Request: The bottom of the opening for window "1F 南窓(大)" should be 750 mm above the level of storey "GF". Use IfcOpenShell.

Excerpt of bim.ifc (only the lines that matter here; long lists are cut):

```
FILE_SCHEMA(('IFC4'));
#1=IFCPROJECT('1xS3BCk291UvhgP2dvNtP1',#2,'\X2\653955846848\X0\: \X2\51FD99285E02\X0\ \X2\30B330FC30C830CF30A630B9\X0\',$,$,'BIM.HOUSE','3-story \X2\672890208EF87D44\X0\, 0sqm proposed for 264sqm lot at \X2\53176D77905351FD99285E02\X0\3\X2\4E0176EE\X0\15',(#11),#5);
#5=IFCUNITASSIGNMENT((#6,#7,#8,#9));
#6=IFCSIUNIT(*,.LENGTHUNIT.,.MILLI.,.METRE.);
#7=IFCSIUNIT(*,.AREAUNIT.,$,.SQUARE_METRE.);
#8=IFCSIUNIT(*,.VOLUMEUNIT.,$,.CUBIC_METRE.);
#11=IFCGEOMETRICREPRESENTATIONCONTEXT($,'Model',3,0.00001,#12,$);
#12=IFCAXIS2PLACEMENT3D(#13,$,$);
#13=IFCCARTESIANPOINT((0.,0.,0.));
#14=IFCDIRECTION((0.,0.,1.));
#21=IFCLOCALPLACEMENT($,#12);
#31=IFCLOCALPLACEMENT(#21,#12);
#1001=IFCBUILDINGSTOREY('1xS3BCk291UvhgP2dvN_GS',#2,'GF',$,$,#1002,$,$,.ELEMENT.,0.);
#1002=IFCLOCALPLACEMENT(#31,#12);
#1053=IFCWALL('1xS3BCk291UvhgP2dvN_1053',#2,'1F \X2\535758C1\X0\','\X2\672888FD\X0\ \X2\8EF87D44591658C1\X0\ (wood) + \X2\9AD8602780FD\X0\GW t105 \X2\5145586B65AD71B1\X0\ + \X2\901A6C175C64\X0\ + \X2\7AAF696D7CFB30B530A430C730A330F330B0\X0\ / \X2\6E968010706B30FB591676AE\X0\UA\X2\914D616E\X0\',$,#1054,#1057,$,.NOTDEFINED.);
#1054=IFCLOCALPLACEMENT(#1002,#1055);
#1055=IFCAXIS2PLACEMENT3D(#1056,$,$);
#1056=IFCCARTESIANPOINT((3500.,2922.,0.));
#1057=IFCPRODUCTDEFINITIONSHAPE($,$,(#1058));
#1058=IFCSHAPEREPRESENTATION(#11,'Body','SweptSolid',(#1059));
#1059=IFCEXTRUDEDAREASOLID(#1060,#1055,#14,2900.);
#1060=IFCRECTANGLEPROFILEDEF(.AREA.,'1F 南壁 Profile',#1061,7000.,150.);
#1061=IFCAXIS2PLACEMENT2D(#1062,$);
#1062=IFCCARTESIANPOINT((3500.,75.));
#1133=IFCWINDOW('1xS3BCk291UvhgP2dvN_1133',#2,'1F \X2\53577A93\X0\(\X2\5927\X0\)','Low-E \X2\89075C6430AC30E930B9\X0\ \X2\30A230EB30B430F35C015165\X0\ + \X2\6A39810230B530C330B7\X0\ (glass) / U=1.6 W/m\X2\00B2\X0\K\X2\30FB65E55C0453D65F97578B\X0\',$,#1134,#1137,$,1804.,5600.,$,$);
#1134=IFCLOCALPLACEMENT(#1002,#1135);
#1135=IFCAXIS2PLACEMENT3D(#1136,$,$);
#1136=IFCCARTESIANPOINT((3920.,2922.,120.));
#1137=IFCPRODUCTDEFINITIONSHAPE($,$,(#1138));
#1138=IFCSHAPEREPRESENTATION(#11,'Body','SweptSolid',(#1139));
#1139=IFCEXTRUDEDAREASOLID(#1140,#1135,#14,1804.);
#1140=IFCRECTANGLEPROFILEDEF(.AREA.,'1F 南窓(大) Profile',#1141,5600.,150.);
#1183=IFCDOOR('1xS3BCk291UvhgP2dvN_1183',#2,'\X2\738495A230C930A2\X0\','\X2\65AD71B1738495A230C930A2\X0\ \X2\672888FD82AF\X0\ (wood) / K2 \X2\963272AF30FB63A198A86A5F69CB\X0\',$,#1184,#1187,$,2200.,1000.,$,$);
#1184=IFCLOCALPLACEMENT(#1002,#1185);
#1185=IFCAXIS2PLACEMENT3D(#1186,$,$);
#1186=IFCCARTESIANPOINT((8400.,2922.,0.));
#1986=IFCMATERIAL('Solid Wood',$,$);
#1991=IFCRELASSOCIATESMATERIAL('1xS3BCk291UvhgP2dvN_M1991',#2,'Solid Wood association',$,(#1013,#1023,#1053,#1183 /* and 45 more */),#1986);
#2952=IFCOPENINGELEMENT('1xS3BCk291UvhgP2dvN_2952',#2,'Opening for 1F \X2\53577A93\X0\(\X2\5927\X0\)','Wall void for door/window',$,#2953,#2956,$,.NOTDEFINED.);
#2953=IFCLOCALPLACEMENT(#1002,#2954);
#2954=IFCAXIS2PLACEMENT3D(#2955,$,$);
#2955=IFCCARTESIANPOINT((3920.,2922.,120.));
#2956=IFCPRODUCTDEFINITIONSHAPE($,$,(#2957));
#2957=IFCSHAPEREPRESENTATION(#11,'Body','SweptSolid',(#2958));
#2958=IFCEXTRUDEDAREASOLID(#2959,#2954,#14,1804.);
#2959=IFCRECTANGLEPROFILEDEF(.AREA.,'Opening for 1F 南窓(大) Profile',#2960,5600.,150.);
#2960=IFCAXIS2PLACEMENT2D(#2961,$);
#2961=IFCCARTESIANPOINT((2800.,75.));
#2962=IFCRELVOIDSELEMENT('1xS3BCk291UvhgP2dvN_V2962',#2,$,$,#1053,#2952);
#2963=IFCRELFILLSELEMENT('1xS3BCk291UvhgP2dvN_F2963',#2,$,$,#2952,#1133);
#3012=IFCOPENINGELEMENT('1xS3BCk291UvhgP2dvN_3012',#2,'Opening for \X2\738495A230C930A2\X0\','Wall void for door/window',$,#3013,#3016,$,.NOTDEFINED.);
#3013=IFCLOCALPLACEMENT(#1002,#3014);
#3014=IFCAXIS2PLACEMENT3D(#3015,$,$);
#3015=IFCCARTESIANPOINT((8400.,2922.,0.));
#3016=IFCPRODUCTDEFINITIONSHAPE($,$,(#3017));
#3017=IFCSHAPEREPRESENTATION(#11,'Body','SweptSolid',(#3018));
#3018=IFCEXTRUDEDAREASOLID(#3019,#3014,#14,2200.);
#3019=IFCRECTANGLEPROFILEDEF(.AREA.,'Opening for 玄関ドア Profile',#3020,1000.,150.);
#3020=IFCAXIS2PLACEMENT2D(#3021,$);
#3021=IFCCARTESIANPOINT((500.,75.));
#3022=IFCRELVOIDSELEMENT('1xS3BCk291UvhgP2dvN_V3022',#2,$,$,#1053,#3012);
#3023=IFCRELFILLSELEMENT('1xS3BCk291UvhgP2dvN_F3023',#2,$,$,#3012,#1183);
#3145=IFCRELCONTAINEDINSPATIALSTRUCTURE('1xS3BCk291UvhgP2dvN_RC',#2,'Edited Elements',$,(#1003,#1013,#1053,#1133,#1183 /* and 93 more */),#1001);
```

```python
import numpy as np
import ifcopenshell
import ifcopenshell.api.geometry
import ifcopenshell.geom
import ifcopenshell.util.element
import ifcopenshell.util.placement
import ifcopenshell.util.shape
import ifcopenshell.util.unit

model = ifcopenshell.open("bim.ifc")
unit_scale = ifcopenshell.util.unit.calculate_unit_scale(model)

window = model.by_guid("1xS3BCk291UvhgP2dvN_1133")
opening = window.FillsVoids[0].RelatingOpeningElement
storey = ifcopenshell.util.element.get_container(window, ifc_class="IfcBuildingStorey")
level = ifcopenshell.util.placement.get_local_placement(storey.ObjectPlacement)[2, 3]

# The opening's origin need not be at the sill, so measure its lowest point.
shape = ifcopenshell.geom.create_shape(ifcopenshell.geom.settings(), opening)
bottom = ifcopenshell.util.shape.get_shape_bottom_elevation(shape, shape.geometry) / unit_scale
dz = level + 0.75 / unit_scale - bottom

shift = np.array([0.0, 0.0, dz])
# The window is not placed relative to its opening, so move both.
for product in (opening, window):
    matrix = ifcopenshell.util.placement.get_local_placement(product.ObjectPlacement)
    matrix[:3, 3] += shift
    ifcopenshell.api.geometry.edit_object_placement(model, product=product, matrix=matrix, is_si=False)

print(f"moved by {dz * unit_scale:+.3f} m")

model.write("bim_edited.ifc")
```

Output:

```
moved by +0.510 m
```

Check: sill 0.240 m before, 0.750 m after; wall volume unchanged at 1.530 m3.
